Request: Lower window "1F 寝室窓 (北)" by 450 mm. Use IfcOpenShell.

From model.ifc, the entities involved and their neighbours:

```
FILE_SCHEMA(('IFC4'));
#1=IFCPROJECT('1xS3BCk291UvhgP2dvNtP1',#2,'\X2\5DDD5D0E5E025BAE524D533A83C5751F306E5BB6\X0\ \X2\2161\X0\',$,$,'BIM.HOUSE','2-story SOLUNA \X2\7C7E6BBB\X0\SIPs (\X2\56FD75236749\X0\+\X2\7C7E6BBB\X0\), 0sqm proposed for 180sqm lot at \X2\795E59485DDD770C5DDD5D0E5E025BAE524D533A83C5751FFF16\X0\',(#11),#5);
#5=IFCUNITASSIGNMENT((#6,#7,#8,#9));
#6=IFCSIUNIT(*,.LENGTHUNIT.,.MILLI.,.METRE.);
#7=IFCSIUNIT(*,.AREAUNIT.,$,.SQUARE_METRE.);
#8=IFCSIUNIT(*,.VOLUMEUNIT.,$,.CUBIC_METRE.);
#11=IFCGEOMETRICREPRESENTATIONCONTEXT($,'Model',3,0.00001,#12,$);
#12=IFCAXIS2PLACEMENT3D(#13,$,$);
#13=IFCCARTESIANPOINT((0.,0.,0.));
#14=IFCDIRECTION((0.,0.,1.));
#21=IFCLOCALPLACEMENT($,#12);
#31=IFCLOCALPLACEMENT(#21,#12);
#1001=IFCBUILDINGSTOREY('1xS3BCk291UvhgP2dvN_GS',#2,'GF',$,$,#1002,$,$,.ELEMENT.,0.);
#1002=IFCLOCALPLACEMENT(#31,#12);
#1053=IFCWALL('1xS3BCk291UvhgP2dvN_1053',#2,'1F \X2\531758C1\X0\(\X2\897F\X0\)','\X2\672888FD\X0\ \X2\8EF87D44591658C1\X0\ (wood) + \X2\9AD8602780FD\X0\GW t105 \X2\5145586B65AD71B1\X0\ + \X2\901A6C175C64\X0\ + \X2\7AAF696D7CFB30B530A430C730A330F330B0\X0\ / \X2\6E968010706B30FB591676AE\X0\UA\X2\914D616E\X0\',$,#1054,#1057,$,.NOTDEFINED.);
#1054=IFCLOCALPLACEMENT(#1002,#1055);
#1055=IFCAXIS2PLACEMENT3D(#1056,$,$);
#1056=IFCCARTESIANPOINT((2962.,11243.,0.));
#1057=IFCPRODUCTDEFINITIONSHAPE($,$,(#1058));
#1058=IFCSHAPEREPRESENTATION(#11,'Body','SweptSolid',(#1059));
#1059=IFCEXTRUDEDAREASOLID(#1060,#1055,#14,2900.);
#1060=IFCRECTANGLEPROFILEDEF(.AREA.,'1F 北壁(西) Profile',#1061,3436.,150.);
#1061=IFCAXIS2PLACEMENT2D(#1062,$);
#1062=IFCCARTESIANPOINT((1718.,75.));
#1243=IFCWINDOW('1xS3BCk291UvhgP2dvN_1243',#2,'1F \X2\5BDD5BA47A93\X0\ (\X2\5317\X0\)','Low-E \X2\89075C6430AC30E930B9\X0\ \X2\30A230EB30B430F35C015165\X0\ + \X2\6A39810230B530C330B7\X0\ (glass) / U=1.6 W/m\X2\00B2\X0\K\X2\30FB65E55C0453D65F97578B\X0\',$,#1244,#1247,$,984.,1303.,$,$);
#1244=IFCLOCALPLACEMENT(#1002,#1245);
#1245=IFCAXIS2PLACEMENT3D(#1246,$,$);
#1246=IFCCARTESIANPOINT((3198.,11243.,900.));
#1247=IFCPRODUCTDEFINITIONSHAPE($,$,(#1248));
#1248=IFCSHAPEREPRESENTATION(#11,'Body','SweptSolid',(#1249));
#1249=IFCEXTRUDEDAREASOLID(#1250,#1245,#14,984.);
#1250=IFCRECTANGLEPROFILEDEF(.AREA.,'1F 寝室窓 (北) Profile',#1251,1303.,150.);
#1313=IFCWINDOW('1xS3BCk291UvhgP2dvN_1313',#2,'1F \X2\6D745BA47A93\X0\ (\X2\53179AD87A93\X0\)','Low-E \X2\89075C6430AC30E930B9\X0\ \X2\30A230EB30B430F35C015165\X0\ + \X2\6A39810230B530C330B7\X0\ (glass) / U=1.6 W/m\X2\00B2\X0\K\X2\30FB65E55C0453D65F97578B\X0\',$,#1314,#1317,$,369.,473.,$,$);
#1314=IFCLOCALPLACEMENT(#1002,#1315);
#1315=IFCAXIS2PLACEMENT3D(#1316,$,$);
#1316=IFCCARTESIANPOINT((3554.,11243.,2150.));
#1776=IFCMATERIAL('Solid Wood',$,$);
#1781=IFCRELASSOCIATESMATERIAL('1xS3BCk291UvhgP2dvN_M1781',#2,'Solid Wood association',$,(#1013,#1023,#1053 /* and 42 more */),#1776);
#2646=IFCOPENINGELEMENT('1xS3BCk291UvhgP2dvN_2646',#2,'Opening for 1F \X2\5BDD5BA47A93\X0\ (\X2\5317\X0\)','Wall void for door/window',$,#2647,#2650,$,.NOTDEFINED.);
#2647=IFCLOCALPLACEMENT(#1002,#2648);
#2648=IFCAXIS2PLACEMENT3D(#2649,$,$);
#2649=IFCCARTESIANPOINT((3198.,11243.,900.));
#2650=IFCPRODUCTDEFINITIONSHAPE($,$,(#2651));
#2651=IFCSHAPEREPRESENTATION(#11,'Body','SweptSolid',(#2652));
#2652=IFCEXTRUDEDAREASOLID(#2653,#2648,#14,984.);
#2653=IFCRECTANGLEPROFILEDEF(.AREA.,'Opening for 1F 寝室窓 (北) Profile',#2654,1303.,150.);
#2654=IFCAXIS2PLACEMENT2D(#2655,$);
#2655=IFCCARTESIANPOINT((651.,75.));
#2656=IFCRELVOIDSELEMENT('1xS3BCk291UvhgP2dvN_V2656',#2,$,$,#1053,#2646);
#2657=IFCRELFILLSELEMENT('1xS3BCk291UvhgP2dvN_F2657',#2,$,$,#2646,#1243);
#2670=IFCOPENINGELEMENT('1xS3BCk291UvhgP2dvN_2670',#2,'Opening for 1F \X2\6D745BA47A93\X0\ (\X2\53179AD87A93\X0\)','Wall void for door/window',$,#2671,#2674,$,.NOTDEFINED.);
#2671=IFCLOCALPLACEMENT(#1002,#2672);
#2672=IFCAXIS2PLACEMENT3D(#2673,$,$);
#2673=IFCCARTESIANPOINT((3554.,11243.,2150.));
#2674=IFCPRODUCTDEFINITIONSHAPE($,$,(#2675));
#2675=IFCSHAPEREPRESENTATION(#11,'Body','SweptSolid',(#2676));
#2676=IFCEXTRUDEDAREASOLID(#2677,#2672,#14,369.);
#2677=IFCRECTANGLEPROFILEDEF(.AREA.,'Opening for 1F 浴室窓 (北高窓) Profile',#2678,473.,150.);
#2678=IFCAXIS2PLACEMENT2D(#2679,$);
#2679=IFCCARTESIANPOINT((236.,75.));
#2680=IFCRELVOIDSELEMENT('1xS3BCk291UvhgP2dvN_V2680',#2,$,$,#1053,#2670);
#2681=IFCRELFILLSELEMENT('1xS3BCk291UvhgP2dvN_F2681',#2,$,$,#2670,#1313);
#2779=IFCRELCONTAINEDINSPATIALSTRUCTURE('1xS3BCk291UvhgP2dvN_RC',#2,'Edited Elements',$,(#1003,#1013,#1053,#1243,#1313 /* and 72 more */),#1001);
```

```python
import numpy as np
import ifcopenshell
import ifcopenshell.api.geometry
import ifcopenshell.util.placement
import ifcopenshell.util.unit

model = ifcopenshell.open("model.ifc")
unit_scale = ifcopenshell.util.unit.calculate_unit_scale(model)

window = model.by_id(1243)
opening = window.FillsVoids[0].RelatingOpeningElement
dz = -0.45 / unit_scale

shift = np.array([0.0, 0.0, dz])
# The window is not placed relative to its opening, so move both.
for product in (opening, window):
    matrix = ifcopenshell.util.placement.get_local_placement(product.ObjectPlacement)
    matrix[:3, 3] += shift
    ifcopenshell.api.geometry.edit_object_placement(model, product=product, matrix=matrix, is_si=False)

print(f"moved by {dz * unit_scale:+.3f} m")

model.write("model_edited.ifc")
```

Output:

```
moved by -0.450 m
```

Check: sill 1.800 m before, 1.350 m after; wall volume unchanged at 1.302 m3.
